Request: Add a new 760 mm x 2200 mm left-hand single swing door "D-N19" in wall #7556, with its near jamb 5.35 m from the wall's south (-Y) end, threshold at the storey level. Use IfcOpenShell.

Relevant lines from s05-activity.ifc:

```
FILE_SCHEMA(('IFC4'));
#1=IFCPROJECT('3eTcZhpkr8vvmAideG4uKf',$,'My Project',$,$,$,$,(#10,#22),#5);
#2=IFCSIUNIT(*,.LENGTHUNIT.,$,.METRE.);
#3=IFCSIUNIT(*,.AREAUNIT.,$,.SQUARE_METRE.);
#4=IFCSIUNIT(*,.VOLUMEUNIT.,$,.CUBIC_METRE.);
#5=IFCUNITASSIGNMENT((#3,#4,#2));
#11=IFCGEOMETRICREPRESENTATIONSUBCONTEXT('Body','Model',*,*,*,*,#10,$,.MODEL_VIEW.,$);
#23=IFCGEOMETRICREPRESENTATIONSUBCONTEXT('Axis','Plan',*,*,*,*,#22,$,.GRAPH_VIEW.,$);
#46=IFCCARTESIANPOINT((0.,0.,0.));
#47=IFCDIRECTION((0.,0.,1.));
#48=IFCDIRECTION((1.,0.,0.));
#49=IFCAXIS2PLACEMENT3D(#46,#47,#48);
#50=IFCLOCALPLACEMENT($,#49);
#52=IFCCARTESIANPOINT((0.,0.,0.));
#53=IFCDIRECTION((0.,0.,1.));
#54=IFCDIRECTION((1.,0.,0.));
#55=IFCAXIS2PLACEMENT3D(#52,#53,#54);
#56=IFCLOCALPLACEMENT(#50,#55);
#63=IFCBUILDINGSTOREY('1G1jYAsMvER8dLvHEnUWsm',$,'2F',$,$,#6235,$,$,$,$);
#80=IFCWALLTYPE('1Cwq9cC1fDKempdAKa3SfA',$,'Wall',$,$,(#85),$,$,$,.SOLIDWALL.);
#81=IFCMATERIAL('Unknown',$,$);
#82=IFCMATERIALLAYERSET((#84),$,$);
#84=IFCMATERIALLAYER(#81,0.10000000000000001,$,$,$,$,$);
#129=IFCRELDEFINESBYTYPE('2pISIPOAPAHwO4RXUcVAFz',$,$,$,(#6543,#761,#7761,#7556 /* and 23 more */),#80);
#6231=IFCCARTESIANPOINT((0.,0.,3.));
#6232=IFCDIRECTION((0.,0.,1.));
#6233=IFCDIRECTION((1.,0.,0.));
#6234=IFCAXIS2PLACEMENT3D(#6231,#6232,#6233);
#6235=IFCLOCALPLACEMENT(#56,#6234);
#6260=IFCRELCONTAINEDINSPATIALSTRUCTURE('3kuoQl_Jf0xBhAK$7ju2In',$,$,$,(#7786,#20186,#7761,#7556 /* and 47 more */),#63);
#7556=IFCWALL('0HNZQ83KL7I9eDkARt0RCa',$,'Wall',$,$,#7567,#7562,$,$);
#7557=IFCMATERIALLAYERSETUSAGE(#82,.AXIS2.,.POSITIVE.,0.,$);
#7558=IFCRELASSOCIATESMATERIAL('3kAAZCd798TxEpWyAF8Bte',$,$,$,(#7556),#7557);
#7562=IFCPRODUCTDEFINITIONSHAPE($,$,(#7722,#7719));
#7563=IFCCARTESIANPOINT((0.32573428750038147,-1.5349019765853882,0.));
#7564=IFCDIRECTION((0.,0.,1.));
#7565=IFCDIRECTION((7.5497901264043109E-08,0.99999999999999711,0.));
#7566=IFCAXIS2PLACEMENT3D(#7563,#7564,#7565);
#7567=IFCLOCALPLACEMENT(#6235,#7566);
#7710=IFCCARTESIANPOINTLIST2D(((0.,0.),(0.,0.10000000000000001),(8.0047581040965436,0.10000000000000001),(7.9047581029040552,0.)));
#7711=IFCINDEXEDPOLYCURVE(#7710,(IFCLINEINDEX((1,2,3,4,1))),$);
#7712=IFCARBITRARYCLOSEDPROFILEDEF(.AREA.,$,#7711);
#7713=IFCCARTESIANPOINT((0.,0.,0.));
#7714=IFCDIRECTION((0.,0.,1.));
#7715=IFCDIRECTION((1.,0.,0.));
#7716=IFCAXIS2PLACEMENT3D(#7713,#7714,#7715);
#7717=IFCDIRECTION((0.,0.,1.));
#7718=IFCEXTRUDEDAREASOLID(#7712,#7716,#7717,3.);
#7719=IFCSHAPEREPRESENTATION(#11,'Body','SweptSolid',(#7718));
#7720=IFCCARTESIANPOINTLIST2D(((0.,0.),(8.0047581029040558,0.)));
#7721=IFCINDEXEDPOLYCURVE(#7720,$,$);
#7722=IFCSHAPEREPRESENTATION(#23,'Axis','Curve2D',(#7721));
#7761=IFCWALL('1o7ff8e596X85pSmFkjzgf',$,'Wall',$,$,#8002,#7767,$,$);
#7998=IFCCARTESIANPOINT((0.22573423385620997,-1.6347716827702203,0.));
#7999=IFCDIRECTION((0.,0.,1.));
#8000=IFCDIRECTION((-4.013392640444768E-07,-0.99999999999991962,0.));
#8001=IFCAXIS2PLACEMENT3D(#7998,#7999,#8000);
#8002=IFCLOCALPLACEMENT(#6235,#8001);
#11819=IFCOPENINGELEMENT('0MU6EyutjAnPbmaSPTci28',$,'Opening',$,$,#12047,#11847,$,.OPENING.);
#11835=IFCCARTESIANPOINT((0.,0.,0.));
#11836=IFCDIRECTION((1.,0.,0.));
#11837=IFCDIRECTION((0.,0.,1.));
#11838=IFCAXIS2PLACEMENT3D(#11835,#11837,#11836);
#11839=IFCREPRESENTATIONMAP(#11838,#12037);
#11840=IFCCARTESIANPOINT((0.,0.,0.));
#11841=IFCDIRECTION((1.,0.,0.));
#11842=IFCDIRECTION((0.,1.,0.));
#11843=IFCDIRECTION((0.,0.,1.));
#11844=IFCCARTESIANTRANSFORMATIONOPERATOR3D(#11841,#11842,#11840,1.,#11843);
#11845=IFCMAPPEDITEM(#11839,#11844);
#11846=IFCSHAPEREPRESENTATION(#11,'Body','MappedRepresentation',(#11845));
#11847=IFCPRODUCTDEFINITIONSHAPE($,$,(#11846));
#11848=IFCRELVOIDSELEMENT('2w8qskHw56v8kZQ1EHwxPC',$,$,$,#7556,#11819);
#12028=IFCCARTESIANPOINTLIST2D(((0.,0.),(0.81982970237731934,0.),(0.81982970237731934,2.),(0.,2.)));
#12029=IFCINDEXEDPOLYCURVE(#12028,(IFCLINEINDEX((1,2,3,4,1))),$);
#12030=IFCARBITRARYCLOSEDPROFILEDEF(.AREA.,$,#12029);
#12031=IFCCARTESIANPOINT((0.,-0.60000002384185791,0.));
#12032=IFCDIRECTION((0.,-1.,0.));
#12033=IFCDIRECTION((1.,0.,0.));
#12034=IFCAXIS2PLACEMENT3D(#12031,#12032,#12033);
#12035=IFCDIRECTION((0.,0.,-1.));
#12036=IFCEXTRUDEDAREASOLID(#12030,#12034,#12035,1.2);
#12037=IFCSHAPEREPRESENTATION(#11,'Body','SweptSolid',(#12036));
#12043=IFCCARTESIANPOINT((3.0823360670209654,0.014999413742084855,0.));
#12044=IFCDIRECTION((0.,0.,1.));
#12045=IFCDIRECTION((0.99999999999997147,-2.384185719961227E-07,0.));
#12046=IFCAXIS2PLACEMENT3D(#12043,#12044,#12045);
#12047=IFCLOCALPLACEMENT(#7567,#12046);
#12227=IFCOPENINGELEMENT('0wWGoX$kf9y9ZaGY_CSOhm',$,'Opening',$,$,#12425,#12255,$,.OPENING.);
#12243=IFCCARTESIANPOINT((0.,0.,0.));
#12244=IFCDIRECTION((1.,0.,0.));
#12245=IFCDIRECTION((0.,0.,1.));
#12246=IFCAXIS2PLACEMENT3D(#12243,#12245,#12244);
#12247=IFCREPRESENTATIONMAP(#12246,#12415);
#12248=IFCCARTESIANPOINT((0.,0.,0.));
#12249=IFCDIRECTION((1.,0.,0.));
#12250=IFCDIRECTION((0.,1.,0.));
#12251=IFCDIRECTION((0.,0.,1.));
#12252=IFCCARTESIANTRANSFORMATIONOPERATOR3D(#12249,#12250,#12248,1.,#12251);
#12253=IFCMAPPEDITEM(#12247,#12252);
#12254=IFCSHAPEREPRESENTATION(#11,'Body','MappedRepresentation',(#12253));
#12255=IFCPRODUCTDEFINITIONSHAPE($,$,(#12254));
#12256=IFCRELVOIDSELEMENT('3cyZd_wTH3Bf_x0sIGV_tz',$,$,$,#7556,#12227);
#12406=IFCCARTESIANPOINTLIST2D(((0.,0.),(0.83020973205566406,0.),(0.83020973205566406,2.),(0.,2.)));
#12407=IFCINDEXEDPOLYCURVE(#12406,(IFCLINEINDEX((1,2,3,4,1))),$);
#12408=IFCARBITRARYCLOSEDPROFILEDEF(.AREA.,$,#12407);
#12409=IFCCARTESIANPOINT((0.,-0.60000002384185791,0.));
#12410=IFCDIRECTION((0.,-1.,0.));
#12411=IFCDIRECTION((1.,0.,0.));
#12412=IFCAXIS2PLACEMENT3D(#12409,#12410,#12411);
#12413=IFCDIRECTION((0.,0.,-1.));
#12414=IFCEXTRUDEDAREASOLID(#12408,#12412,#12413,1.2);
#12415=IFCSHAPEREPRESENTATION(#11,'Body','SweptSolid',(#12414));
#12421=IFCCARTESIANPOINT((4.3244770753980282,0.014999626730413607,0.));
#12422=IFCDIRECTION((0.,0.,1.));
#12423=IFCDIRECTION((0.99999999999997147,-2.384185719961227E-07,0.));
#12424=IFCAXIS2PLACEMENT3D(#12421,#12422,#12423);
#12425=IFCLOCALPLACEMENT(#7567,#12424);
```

```python
import numpy as np
import ifcopenshell
import ifcopenshell.api.feature
import ifcopenshell.api.geometry
import ifcopenshell.api.root
import ifcopenshell.api.spatial
import ifcopenshell.geom
import ifcopenshell.util.element
import ifcopenshell.util.placement
import ifcopenshell.util.representation
import ifcopenshell.util.shape
import ifcopenshell.util.unit

model = ifcopenshell.open("s05-activity.ifc")
unit_scale = ifcopenshell.util.unit.calculate_unit_scale(model)
settings = ifcopenshell.geom.settings()


def volume(element):
    """Net volume in cubic metres, openings subtracted."""
    shape = ifcopenshell.geom.create_shape(settings, element)
    return ifcopenshell.util.shape.get_volume(shape.geometry)


wall = model.by_guid("0HNZQ83KL7I9eDkARt0RCa")
storey = ifcopenshell.util.element.get_container(wall, ifc_class="IfcBuildingStorey")
context = ifcopenshell.util.representation.get_context(model, "Model", "Body", "MODEL_VIEW")
before = volume(wall)

width, height, from_end, sill = 0.76, 2.2, 5.35, 0.0  # metres

# The wall runs along its own X axis, and the end named is its -X end.
wall_shape = ifcopenshell.geom.create_shape(settings, wall)
x, y, z = ifcopenshell.util.shape.get_vertices(wall_shape.geometry).T
start = x.min() + from_end
face, thickness = float(y.min()), float(y.max() - y.min())
wall_matrix = ifcopenshell.util.placement.get_local_placement(wall.ObjectPlacement)
level = ifcopenshell.util.placement.get_local_placement(storey.ObjectPlacement)[2, 3]


def in_wall(x, y):
    """Placement at x, y metres in the wall's axes, at sill height."""
    matrix = wall_matrix.copy()
    matrix[:, 3] = wall_matrix @ np.array([x / unit_scale, y / unit_scale, 0.0, 1.0])
    matrix[2, 3] = level + sill / unit_scale
    return matrix


# Opening: a box that overshoots both wall faces by 50 mm.
opening = ifcopenshell.api.root.create_entity(model, ifc_class="IfcOpeningElement", predefined_type="OPENING")
box = ifcopenshell.api.geometry.add_wall_representation(
    model, context=context, length=width, height=height, thickness=thickness + 0.1
)
ifcopenshell.api.geometry.assign_representation(model, product=opening, representation=box)
ifcopenshell.api.geometry.edit_object_placement(model, product=opening, matrix=in_wall(start, face - 0.05), is_si=False)
ifcopenshell.api.feature.add_feature(model, feature=opening, element=wall)

door = ifcopenshell.api.root.create_entity(model, ifc_class="IfcDoor", name="D-N19", predefined_type="DOOR")
door.OverallWidth, door.OverallHeight = width / unit_scale, height / unit_scale
door.OperationType = "SINGLE_SWING_LEFT"
body = ifcopenshell.api.geometry.add_door_representation(
    model,
    context=context,
    overall_width=door.OverallWidth,
    overall_height=door.OverallHeight,
    operation_type="SINGLE_SWING_LEFT",
    lining_properties={"LiningDepth": thickness / unit_scale, "ThresholdDepth": thickness / unit_scale},
)
ifcopenshell.api.geometry.assign_representation(model, product=door, representation=body)
ifcopenshell.api.spatial.assign_container(model, products=[door], relating_structure=storey)
ifcopenshell.api.feature.add_filling(model, opening=opening, element=door)

# The lining spans the wall, so the door starts at the wall face.
ifcopenshell.api.geometry.edit_object_placement(model, product=door, matrix=in_wall(start, face), is_si=False)

after = volume(wall)

print(f"wall volume {before:.3f} -> {after:.3f} m3")

model.write("s05-activity_v2.ifc")
```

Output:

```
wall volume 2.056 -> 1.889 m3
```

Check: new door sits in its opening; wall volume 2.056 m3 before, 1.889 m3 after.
